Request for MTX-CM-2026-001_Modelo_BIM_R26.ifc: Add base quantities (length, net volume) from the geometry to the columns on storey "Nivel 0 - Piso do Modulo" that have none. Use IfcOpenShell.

First a look at what the model holds.

```python
import ifcopenshell
import ifcopenshell.util.element
import ifcopenshell.util.unit

model = ifcopenshell.open("MTX-CM-2026-001_Modelo_BIM_R26.ifc")
print(model.schema)
for unit_type in ("LENGTHUNIT", "AREAUNIT", "VOLUMEUNIT"):
    print(unit_type, ifcopenshell.util.unit.calculate_unit_scale(model, unit_type))
storey = next(s for s in model.by_type("IfcBuildingStorey") if s.Name == "Nivel 0 - Piso do Modulo")
columns = [e for e in ifcopenshell.util.element.get_decomposition(storey) if e.is_a("IfcColumn")]
for e in sorted(columns, key=lambda e: e.id()):
    print(e.id(), e.is_a(), e.Name, list(ifcopenshell.util.element.get_psets(e, qtos_only=True)), sep=" | ")
```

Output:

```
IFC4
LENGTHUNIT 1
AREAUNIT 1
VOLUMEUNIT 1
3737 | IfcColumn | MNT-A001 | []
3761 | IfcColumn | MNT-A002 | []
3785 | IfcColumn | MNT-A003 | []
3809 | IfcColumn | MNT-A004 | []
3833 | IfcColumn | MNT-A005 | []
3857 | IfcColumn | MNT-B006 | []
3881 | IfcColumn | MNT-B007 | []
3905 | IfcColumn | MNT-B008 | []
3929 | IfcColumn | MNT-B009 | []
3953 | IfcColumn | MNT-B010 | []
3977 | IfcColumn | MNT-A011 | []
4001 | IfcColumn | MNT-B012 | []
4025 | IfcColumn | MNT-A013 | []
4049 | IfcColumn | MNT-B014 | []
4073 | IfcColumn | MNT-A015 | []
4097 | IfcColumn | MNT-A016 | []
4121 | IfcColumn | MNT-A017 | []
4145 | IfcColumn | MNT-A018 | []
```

```python
import ifcopenshell
import ifcopenshell.api.pset
import ifcopenshell.geom
import ifcopenshell.util.element
import ifcopenshell.util.shape
import ifcopenshell.util.unit

model = ifcopenshell.open("MTX-CM-2026-001_Modelo_BIM_R26.ifc")
unit_scale = ifcopenshell.util.unit.calculate_unit_scale(model)
volume_scale = ifcopenshell.util.unit.calculate_unit_scale(model, "VOLUMEUNIT")
settings = ifcopenshell.geom.settings()

storey = next(s for s in model.by_type("IfcBuildingStorey") if s.Name == "Nivel 0 - Piso do Modulo")
columns = [e for e in ifcopenshell.util.element.get_decomposition(storey) if e.is_a("IfcColumn")]

for e in sorted(columns, key=lambda e: e.id()):
    if ifcopenshell.util.element.get_psets(e, qtos_only=True, should_inherit=False):
        continue
    # Geometry comes back in metres, in the element's own axes.
    shape = ifcopenshell.geom.create_shape(settings, e)
    values = {
        "Length": ifcopenshell.util.shape.get_z(shape.geometry) / unit_scale,
        "NetVolume": ifcopenshell.util.shape.get_volume(shape.geometry) / volume_scale,
    }
    qto = ifcopenshell.api.pset.add_qto(model, product=e, name="Qto_ColumnBaseQuantities")
    ifcopenshell.api.pset.edit_qto(model, qto=qto, properties=values)
    print(e.id(), {k: round(v, 3) for k, v in values.items()})

model.write("MTX-CM-2026-001_Modelo_BIM_R26-out.ifc")
```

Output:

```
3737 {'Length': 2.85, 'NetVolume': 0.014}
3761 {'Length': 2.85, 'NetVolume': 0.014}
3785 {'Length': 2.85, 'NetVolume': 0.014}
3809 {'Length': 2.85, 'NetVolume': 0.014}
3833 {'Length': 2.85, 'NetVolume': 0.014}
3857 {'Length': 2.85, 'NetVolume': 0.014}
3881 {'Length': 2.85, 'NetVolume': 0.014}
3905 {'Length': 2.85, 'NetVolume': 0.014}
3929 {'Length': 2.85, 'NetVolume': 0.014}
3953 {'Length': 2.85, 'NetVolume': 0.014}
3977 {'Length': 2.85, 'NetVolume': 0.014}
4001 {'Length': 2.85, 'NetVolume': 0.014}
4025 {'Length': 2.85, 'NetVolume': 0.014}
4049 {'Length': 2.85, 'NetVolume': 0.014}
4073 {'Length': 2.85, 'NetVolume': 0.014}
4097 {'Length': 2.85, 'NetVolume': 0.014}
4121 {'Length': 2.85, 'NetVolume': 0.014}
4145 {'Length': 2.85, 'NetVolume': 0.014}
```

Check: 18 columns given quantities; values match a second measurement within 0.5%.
